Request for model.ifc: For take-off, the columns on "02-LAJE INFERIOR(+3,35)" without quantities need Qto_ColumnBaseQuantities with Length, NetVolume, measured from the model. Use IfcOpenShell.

First a look at what the model holds.

```python
import ifcopenshell
import ifcopenshell.util.element
import ifcopenshell.util.unit

model = ifcopenshell.open("model.ifc")
print(model.schema)
for unit_type in ("LENGTHUNIT", "AREAUNIT", "VOLUMEUNIT"):
    print(unit_type, ifcopenshell.util.unit.calculate_unit_scale(model, unit_type))
storey = next(s for s in model.by_type("IfcBuildingStorey") if s.Name == "02-LAJE INFERIOR(+3,35)")
columns = [e for e in ifcopenshell.util.element.get_decomposition(storey) if e.is_a("IfcColumn")]
for e in sorted(columns, key=lambda e: e.id()):
    print(e.id(), e.is_a(), e.Name, list(ifcopenshell.util.element.get_psets(e, qtos_only=True)), sep=" | ")
```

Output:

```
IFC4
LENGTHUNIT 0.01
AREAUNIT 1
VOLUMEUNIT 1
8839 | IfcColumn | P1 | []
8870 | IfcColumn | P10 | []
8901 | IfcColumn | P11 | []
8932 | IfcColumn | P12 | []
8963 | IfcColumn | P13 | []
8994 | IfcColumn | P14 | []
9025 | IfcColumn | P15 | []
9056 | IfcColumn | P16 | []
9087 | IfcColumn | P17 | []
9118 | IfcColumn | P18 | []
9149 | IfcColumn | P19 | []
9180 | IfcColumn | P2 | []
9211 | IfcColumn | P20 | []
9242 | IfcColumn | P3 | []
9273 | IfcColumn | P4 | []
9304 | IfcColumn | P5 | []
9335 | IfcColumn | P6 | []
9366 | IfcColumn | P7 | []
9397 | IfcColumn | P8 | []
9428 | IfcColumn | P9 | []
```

```python
import ifcopenshell
import ifcopenshell.api.pset
import ifcopenshell.geom
import ifcopenshell.util.element
import ifcopenshell.util.shape
import ifcopenshell.util.unit

model = ifcopenshell.open("model.ifc")
unit_scale = ifcopenshell.util.unit.calculate_unit_scale(model)
volume_scale = ifcopenshell.util.unit.calculate_unit_scale(model, "VOLUMEUNIT")
settings = ifcopenshell.geom.settings()

storey = next(s for s in model.by_type("IfcBuildingStorey") if s.Name == "02-LAJE INFERIOR(+3,35)")
columns = [e for e in ifcopenshell.util.element.get_decomposition(storey) if e.is_a("IfcColumn")]

for e in sorted(columns, key=lambda e: e.id()):
    if ifcopenshell.util.element.get_psets(e, qtos_only=True, should_inherit=False):
        continue
    # Geometry comes back in metres, in the element's own axes.
    shape = ifcopenshell.geom.create_shape(settings, e)
    values = {
        "Length": ifcopenshell.util.shape.get_z(shape.geometry) / unit_scale,
        "NetVolume": ifcopenshell.util.shape.get_volume(shape.geometry) / volume_scale,
    }
    qto = ifcopenshell.api.pset.add_qto(model, product=e, name="Qto_ColumnBaseQuantities")
    ifcopenshell.api.pset.edit_qto(model, qto=qto, properties=values)
    print(e.id(), {k: round(v, 3) for k, v in values.items()})

model.write("model_rev.ifc")
```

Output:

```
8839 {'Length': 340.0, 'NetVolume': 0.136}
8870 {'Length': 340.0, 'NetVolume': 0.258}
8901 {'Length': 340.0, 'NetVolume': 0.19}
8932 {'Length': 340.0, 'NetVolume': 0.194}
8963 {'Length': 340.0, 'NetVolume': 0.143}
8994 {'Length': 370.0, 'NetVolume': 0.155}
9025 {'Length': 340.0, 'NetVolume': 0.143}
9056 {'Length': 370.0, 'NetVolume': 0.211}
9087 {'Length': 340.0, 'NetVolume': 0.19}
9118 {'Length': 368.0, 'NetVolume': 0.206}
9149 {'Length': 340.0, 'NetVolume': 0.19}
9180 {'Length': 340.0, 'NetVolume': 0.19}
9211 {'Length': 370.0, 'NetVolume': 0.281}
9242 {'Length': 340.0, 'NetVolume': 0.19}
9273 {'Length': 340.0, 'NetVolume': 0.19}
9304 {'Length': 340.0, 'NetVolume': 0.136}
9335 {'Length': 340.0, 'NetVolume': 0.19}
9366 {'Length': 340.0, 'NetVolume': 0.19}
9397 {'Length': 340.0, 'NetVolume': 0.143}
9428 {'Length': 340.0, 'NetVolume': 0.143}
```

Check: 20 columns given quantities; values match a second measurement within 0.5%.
